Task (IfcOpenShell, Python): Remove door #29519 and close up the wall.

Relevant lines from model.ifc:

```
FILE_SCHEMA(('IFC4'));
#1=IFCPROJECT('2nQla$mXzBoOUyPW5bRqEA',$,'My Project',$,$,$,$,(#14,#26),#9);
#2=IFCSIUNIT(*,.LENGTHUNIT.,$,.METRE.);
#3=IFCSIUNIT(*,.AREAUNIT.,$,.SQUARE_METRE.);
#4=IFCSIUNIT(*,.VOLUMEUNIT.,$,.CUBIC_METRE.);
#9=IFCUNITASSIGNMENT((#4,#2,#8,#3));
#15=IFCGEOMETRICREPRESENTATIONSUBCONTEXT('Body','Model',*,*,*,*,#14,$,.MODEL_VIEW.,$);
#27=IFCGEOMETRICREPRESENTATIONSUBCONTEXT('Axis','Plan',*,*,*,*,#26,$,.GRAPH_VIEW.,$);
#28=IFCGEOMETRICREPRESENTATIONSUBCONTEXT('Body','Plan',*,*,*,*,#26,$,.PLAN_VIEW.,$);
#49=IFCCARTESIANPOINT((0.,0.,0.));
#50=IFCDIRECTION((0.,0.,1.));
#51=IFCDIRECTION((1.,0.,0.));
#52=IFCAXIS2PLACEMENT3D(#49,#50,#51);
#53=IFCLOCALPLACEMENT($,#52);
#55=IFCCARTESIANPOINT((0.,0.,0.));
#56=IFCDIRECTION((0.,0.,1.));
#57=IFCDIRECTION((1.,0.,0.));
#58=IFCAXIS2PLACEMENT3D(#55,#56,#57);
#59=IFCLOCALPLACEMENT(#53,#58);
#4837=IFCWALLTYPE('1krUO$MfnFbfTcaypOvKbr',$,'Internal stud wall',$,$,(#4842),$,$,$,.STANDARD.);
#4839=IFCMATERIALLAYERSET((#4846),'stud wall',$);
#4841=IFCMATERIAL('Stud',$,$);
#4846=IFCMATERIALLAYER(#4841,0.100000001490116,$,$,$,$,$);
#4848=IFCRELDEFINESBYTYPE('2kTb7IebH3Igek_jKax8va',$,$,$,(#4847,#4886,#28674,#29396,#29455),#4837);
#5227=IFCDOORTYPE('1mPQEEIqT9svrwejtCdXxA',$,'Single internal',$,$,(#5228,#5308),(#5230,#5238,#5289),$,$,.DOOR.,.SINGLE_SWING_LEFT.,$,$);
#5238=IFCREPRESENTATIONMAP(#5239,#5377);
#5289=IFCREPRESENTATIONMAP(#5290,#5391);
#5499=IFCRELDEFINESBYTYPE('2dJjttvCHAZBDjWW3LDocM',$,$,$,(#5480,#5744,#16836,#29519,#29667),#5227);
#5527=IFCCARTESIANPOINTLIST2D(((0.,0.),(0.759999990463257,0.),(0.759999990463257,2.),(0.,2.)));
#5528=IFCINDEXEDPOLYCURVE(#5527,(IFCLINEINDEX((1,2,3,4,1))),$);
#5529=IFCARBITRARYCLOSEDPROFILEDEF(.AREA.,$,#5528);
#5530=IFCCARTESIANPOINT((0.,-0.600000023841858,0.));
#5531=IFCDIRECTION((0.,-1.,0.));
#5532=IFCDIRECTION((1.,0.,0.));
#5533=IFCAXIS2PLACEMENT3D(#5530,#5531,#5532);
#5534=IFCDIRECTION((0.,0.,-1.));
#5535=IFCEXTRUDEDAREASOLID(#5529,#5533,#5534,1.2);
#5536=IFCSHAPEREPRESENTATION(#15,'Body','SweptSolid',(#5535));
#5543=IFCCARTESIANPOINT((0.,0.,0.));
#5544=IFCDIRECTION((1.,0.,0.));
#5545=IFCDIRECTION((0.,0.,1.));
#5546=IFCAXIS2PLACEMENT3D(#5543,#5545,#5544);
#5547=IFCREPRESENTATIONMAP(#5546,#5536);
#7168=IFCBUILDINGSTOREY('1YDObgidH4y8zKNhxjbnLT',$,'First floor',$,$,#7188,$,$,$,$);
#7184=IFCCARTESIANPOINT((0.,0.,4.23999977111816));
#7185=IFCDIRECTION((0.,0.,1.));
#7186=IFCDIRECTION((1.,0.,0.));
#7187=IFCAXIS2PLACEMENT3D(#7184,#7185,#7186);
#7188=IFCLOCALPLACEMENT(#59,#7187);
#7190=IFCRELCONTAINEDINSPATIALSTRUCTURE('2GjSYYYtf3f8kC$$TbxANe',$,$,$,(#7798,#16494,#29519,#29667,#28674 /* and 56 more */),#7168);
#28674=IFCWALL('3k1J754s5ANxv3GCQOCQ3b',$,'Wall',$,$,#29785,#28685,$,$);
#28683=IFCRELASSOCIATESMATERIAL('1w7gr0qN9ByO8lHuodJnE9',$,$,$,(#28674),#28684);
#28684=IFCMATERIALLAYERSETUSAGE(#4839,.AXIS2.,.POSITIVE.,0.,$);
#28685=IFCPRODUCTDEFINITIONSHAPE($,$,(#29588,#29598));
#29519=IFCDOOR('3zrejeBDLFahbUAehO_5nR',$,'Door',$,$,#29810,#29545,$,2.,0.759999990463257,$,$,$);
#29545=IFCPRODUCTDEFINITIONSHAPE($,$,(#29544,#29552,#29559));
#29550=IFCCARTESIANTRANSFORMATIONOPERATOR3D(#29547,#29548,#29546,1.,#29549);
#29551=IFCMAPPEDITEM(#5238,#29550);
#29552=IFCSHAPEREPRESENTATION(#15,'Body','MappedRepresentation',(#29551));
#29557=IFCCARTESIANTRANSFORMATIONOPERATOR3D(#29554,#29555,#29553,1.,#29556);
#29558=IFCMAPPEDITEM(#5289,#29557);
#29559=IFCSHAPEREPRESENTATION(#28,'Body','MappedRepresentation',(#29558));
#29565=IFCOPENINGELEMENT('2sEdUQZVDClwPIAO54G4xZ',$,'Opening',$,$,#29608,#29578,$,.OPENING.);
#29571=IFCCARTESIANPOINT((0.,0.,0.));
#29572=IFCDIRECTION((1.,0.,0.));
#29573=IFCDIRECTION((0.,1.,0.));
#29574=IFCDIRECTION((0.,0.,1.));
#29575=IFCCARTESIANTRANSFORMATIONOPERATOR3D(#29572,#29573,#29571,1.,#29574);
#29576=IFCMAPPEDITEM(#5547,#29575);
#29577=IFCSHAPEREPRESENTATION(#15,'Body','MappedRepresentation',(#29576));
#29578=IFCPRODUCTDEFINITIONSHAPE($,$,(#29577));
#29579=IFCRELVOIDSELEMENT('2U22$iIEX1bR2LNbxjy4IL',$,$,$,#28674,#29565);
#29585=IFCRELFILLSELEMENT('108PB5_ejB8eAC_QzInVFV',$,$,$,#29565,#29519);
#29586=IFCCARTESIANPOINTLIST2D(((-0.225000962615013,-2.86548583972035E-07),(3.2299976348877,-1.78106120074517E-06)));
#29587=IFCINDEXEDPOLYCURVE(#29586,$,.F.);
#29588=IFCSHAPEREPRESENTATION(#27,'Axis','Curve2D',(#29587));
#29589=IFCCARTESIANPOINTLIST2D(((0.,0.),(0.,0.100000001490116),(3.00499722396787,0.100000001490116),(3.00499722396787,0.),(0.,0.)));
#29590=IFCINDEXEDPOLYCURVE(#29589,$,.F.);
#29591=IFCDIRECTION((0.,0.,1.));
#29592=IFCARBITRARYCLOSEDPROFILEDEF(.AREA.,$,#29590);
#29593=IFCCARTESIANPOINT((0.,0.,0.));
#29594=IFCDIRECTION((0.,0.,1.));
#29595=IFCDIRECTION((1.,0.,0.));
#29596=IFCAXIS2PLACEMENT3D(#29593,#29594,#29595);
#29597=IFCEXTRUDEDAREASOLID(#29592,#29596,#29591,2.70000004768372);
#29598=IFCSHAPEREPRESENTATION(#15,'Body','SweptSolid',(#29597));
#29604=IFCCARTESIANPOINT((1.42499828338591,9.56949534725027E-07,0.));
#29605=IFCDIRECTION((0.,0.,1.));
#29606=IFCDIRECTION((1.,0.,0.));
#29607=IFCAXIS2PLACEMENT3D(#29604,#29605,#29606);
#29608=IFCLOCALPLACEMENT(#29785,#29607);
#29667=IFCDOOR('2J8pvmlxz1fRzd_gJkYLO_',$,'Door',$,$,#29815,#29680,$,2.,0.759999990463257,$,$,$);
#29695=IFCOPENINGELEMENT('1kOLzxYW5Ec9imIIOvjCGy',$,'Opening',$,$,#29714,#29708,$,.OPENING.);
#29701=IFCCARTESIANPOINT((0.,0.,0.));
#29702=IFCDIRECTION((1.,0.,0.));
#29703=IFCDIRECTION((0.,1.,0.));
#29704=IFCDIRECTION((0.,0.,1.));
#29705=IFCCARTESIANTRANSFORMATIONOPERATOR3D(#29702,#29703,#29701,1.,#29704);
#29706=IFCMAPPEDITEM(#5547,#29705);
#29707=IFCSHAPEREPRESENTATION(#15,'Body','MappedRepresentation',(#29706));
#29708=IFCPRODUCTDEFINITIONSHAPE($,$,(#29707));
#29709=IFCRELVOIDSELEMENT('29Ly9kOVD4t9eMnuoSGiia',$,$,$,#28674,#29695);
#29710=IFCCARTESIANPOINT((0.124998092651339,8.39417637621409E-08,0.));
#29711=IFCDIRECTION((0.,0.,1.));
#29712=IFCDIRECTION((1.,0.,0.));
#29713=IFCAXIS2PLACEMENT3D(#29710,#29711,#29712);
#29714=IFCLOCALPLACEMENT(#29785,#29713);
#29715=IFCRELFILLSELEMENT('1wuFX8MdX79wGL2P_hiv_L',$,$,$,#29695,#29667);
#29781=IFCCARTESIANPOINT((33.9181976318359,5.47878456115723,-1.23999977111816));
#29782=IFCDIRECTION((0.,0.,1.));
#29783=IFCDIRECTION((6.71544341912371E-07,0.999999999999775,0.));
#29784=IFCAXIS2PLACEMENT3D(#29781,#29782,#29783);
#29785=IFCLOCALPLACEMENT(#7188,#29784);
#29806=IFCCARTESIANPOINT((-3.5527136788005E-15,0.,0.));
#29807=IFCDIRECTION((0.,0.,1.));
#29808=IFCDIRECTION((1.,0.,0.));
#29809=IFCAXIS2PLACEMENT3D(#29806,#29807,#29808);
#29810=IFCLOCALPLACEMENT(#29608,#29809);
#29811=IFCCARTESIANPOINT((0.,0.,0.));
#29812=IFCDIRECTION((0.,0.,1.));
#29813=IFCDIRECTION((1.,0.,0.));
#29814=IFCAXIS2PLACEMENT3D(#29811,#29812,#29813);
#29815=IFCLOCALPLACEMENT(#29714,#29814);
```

```python
import ifcopenshell
import ifcopenshell.api.feature
import ifcopenshell.api.root
import ifcopenshell.geom
import ifcopenshell.util.shape

model = ifcopenshell.open("model.ifc")
settings = ifcopenshell.geom.settings()


def volume(element):
    """Net volume in cubic metres, openings subtracted."""
    shape = ifcopenshell.geom.create_shape(settings, element)
    return ifcopenshell.util.shape.get_volume(shape.geometry)


door = model.by_guid("3zrejeBDLFahbUAehO_5nR")
opening = door.FillsVoids[0].RelatingOpeningElement
wall = opening.VoidsElements[0].RelatingBuildingElement
before = volume(wall)

ifcopenshell.api.root.remove_product(model, product=door)
ifcopenshell.api.feature.remove_feature(model, feature=opening)

after = volume(wall)

print(f"wall volume {before:.3f} -> {after:.3f} m3")

model.write("model_edited.ifc")
```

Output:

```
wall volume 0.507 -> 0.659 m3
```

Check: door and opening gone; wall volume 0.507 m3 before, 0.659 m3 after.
